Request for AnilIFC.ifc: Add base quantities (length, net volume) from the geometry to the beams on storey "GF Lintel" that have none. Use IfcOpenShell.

First a look at what the model holds.

```python
import ifcopenshell
import ifcopenshell.util.element
import ifcopenshell.util.unit

model = ifcopenshell.open("AnilIFC.ifc")
print(model.schema)
for unit_type in ("LENGTHUNIT", "AREAUNIT", "VOLUMEUNIT"):
    print(unit_type, ifcopenshell.util.unit.calculate_unit_scale(model, unit_type))
storey = next(s for s in model.by_type("IfcBuildingStorey") if s.Name == "GF Lintel")
beams = [e for e in ifcopenshell.util.element.get_decomposition(storey) if e.is_a("IfcBeam")]
for e in sorted(beams, key=lambda e: e.id()):
    print(e.id(), e.is_a(), e.Name, list(ifcopenshell.util.element.get_psets(e, qtos_only=True)), sep=" | ")
```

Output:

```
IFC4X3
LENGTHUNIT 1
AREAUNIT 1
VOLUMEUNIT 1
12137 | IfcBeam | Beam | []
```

```python
import ifcopenshell
import ifcopenshell.api.pset
import ifcopenshell.geom
import ifcopenshell.util.element
import ifcopenshell.util.shape
import ifcopenshell.util.unit

model = ifcopenshell.open("AnilIFC.ifc")
unit_scale = ifcopenshell.util.unit.calculate_unit_scale(model)
volume_scale = ifcopenshell.util.unit.calculate_unit_scale(model, "VOLUMEUNIT")
settings = ifcopenshell.geom.settings()

storey = next(s for s in model.by_type("IfcBuildingStorey") if s.Name == "GF Lintel")
beams = [e for e in ifcopenshell.util.element.get_decomposition(storey) if e.is_a("IfcBeam")]

for e in sorted(beams, key=lambda e: e.id()):
    if ifcopenshell.util.element.get_psets(e, qtos_only=True, should_inherit=False):
        continue
    # Geometry comes back in metres, in the element's own axes.
    shape = ifcopenshell.geom.create_shape(settings, e)
    values = {
        "Length": ifcopenshell.util.shape.get_max_xyz(shape.geometry) / unit_scale,
        "NetVolume": ifcopenshell.util.shape.get_volume(shape.geometry) / volume_scale,
    }
    qto = ifcopenshell.api.pset.add_qto(model, product=e, name="Qto_BeamBaseQuantities")
    ifcopenshell.api.pset.edit_qto(model, qto=qto, properties=values)
    print(e.id(), {k: round(v, 3) for k, v in values.items()})

model.write("AnilIFC_edited.ifc")
```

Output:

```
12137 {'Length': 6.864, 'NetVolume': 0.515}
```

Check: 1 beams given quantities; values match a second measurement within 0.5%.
